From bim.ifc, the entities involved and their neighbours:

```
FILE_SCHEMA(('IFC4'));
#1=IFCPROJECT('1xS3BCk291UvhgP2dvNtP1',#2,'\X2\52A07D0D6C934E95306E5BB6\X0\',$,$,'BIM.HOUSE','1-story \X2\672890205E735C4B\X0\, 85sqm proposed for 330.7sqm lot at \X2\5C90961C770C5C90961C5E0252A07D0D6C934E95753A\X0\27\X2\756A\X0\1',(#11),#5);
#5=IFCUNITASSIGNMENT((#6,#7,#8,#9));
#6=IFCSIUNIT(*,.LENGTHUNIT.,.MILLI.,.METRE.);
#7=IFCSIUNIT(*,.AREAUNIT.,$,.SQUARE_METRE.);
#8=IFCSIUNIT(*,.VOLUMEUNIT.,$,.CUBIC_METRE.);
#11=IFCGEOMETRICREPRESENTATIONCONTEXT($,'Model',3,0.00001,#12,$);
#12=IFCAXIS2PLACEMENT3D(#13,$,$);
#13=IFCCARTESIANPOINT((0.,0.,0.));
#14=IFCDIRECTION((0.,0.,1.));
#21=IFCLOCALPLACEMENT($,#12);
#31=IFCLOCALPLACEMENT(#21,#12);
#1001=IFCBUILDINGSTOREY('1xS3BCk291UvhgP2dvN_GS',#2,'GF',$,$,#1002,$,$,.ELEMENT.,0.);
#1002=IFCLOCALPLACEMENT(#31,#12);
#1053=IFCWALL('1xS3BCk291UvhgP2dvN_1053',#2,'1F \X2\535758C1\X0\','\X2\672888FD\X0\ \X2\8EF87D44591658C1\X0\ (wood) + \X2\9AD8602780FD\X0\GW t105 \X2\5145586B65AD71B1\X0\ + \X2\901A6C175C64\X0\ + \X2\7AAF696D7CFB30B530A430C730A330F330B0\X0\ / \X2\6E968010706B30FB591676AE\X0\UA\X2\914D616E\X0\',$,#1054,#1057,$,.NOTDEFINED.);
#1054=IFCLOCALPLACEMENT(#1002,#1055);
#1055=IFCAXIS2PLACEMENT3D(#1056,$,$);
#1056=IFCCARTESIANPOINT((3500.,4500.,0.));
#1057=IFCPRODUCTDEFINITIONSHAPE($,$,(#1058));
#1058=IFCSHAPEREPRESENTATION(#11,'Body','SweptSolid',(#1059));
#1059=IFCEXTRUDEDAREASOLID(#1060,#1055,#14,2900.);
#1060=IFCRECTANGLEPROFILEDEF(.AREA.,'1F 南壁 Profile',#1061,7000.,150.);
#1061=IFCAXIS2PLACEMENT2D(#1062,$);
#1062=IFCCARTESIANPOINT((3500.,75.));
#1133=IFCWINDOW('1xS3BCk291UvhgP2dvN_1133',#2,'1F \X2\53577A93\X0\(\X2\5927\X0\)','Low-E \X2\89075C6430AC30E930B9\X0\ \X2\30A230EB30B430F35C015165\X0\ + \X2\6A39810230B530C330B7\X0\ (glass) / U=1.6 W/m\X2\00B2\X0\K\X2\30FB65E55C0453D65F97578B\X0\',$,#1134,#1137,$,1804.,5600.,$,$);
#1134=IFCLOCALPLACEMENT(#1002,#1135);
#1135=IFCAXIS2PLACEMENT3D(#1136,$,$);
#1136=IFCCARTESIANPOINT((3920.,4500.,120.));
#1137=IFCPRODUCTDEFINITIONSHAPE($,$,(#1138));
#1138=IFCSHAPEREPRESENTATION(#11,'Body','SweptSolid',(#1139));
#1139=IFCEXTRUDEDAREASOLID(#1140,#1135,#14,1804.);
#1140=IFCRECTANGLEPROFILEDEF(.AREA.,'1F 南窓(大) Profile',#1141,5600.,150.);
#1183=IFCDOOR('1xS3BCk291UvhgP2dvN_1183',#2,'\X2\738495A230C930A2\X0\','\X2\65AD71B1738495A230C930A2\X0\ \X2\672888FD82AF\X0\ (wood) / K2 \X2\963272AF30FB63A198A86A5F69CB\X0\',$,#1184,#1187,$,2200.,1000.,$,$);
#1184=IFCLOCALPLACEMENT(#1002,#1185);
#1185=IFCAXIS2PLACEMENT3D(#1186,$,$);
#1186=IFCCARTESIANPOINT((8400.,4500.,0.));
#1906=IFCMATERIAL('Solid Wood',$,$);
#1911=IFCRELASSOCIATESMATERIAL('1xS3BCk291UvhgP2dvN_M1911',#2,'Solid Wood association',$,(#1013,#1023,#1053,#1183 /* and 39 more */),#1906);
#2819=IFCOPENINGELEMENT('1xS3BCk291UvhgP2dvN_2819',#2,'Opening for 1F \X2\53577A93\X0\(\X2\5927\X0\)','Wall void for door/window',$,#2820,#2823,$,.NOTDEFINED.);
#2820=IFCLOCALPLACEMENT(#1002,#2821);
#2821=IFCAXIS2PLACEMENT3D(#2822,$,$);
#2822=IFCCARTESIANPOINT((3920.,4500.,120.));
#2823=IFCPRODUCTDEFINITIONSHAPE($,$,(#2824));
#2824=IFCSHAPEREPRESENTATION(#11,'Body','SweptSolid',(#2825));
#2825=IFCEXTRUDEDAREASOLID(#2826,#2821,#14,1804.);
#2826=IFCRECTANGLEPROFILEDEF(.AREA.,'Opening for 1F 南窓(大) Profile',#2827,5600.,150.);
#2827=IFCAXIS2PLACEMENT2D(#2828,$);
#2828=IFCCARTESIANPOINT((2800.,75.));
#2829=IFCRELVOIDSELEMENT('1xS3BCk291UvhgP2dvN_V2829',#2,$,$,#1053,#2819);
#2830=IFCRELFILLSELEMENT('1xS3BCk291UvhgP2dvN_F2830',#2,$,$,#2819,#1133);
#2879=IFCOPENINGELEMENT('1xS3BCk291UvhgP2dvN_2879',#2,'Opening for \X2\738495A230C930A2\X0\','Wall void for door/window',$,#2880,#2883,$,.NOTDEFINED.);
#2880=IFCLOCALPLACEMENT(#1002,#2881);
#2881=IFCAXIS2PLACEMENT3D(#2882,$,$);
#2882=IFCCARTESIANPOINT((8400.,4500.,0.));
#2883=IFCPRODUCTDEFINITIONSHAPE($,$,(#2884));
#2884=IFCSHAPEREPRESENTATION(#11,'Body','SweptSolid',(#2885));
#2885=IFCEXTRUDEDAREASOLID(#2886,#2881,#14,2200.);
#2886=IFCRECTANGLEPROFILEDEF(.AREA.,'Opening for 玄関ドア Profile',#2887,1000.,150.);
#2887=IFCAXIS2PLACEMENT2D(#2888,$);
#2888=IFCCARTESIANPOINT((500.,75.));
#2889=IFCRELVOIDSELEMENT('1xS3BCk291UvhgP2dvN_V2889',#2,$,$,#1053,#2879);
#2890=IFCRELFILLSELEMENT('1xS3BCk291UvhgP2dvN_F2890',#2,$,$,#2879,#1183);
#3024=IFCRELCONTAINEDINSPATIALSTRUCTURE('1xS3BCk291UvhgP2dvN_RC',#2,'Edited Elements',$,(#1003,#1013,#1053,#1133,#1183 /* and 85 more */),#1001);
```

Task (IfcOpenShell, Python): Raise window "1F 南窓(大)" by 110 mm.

```python
import numpy as np
import ifcopenshell
import ifcopenshell.api.geometry
import ifcopenshell.util.placement
import ifcopenshell.util.unit

model = ifcopenshell.open("bim.ifc")
unit_scale = ifcopenshell.util.unit.calculate_unit_scale(model)

window = model.by_guid("1xS3BCk291UvhgP2dvN_1133")
opening = window.FillsVoids[0].RelatingOpeningElement
dz = 110.0

shift = np.array([0.0, 0.0, dz])
# The window is not placed relative to its opening, so move both.
for product in (opening, window):
    matrix = ifcopenshell.util.placement.get_local_placement(product.ObjectPlacement)
    matrix[:3, 3] += shift
    ifcopenshell.api.geometry.edit_object_placement(model, product=product, matrix=matrix, is_si=False)

print(f"moved by {dz * unit_scale:+.3f} m")

model.write("bim_updated.ifc")
```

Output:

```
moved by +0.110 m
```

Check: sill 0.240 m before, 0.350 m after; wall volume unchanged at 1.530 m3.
